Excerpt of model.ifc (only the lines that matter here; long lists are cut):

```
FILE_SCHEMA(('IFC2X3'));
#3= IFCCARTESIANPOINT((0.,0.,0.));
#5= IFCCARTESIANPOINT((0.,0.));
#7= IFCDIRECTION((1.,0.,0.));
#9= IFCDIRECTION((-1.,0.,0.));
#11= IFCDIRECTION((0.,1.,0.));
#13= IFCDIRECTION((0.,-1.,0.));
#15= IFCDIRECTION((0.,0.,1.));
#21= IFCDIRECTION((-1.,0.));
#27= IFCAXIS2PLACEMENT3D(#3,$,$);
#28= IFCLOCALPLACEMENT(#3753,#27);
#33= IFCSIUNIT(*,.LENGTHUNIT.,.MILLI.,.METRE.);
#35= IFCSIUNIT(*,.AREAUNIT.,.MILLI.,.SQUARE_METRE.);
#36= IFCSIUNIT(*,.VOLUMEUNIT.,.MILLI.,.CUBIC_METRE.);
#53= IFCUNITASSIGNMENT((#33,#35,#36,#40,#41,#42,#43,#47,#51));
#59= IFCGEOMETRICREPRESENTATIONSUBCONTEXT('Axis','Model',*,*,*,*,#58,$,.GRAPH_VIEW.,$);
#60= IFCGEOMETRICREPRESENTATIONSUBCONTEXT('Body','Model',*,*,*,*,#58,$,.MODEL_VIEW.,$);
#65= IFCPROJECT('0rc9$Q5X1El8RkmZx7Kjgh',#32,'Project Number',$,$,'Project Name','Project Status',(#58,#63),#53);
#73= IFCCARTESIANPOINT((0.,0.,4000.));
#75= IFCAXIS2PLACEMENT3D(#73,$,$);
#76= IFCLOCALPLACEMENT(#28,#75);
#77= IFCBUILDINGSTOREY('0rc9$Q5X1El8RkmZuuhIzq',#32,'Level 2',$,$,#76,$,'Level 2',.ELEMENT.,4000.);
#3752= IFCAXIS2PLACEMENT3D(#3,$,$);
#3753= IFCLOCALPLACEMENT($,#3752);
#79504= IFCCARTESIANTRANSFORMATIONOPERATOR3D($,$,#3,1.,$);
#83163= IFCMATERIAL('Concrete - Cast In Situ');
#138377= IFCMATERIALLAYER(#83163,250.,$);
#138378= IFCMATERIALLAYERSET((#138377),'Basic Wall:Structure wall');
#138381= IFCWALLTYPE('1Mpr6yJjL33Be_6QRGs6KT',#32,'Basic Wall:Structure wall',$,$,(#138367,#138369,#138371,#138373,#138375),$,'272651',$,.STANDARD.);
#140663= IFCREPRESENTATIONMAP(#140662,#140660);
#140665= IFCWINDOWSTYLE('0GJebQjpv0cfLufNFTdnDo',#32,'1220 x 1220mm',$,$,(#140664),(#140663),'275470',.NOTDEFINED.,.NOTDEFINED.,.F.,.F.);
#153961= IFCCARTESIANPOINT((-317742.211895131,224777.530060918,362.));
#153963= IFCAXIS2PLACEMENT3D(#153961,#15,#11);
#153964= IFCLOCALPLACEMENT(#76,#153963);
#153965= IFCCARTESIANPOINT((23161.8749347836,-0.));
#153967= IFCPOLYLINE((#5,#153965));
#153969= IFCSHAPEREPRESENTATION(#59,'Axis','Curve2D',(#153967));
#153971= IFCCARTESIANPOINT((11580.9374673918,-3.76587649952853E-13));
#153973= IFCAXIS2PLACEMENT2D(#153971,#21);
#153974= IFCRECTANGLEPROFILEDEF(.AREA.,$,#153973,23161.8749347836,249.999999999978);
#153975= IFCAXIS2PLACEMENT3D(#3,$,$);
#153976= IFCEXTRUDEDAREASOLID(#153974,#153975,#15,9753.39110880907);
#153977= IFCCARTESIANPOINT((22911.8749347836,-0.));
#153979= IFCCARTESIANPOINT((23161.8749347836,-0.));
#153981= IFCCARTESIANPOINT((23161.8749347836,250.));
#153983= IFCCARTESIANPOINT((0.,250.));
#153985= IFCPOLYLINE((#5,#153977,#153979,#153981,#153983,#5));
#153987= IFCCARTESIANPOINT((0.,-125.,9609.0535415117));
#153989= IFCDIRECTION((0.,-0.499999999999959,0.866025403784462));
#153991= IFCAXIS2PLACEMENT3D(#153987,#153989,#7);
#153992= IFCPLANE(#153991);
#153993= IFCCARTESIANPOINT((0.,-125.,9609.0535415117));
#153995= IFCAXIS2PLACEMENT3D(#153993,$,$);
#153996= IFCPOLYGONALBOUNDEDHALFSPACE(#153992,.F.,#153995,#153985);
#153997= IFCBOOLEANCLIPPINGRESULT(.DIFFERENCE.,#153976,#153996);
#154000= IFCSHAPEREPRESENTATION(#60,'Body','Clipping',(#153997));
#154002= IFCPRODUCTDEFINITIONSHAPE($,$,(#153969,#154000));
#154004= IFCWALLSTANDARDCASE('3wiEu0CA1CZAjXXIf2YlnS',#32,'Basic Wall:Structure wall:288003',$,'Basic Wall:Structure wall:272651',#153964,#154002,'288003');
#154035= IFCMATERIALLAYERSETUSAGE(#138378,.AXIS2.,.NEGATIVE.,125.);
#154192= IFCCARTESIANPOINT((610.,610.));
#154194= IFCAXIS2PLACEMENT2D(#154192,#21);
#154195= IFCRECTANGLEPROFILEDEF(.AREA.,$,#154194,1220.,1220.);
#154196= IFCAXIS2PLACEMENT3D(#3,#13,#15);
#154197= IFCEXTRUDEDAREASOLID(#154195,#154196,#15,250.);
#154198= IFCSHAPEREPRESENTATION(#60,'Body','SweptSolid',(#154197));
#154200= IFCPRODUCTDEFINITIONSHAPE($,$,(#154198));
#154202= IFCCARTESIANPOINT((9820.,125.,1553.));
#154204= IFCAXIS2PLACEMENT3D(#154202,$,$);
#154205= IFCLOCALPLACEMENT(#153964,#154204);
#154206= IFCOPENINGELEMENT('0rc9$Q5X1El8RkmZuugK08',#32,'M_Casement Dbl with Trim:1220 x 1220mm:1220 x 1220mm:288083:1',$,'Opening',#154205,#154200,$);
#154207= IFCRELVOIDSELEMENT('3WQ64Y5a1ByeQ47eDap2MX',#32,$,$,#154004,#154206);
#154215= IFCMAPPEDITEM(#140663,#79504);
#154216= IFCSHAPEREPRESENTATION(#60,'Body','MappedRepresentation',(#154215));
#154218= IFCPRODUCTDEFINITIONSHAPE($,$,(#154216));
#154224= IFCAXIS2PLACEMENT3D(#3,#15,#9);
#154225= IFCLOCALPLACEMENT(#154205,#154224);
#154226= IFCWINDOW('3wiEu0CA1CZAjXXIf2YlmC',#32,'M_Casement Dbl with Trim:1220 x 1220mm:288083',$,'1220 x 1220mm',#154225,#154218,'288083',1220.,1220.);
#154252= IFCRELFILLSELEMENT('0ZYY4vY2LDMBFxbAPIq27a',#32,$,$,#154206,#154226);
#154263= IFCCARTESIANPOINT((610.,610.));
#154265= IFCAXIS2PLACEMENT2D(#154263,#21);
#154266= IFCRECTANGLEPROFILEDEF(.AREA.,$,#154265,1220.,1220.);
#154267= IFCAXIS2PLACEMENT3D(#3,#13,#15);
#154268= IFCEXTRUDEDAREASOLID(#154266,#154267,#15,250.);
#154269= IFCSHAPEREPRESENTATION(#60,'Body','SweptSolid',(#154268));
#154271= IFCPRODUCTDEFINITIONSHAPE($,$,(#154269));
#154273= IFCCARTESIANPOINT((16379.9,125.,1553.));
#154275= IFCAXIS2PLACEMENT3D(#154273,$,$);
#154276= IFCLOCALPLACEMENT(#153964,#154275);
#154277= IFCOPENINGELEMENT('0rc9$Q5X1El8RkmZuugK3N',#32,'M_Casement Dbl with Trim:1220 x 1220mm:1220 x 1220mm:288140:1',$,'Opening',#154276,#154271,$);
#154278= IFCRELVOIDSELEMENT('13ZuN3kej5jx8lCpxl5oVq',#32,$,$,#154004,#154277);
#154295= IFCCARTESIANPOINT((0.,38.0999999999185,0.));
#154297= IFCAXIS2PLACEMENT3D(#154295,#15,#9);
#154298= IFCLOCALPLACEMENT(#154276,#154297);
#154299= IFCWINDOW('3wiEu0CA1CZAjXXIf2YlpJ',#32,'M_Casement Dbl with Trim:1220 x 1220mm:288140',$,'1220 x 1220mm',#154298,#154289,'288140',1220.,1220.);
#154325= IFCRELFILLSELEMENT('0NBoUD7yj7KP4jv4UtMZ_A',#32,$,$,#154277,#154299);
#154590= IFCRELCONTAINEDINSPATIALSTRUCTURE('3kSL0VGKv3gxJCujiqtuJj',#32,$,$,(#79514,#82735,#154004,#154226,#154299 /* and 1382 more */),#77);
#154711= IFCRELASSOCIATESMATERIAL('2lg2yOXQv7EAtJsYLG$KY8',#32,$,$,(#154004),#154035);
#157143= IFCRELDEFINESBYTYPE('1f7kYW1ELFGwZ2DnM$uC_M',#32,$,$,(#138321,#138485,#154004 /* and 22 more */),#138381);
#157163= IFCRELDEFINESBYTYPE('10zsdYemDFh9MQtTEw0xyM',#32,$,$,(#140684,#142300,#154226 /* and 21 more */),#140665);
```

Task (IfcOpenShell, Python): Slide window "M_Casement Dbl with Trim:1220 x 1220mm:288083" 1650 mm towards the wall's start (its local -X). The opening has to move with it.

```python
import ifcopenshell
import ifcopenshell.api.geometry
import ifcopenshell.util.placement
import ifcopenshell.util.unit

model = ifcopenshell.open("model.ifc")
unit_scale = ifcopenshell.util.unit.calculate_unit_scale(model)

window = model.by_guid("3wiEu0CA1CZAjXXIf2YlmC")
opening = window.FillsVoids[0].RelatingOpeningElement
wall = opening.VoidsElements[0].RelatingBuildingElement

wall_matrix = ifcopenshell.util.placement.get_local_placement(wall.ObjectPlacement)
shift = wall_matrix[:3, 0] * -1.65 / unit_scale
before = ifcopenshell.util.placement.get_local_placement(window.ObjectPlacement)[:3, 3].copy()

# The window is placed relative to its opening, so it follows when the opening moves.
matrix = ifcopenshell.util.placement.get_local_placement(opening.ObjectPlacement)
matrix[:3, 3] += shift
ifcopenshell.api.geometry.edit_object_placement(
    model, product=opening, matrix=matrix, is_si=False, should_transform_children=True
)

after = ifcopenshell.util.placement.get_local_placement(window.ObjectPlacement)[:3, 3]
print("window moved by", (after - before).round(3) + 0.0)

model.write("model_v2.ifc")
```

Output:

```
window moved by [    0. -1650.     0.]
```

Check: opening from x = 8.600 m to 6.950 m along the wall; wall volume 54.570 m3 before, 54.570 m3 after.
